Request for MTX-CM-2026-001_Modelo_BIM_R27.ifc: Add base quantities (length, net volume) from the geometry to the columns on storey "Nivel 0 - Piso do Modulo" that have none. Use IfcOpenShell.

First a look at what the model holds.

```python
import ifcopenshell
import ifcopenshell.util.element
import ifcopenshell.util.unit

model = ifcopenshell.open("MTX-CM-2026-001_Modelo_BIM_R27.ifc")
print(model.schema)
for unit_type in ("LENGTHUNIT", "AREAUNIT", "VOLUMEUNIT"):
    print(unit_type, ifcopenshell.util.unit.calculate_unit_scale(model, unit_type))
storey = next(s for s in model.by_type("IfcBuildingStorey") if s.Name == "Nivel 0 - Piso do Modulo")
columns = [e for e in ifcopenshell.util.element.get_decomposition(storey) if e.is_a("IfcColumn")]
for e in sorted(columns, key=lambda e: e.id()):
    print(e.id(), e.is_a(), e.Name, list(ifcopenshell.util.element.get_psets(e, qtos_only=True)), sep=" | ")
```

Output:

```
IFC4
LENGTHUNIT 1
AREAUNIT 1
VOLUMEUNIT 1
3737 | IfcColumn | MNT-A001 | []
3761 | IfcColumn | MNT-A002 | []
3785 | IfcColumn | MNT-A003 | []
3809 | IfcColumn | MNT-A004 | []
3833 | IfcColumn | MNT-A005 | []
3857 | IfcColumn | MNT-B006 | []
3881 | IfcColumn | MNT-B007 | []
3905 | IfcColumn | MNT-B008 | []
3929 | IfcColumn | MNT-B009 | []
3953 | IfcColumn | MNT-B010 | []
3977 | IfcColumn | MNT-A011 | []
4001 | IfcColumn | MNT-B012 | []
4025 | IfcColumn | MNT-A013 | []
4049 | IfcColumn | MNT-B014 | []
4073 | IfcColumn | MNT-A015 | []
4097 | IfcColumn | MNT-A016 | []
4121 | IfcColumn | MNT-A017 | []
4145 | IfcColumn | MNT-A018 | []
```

```python
import ifcopenshell
import ifcopenshell.api.pset
import ifcopenshell.geom
import ifcopenshell.util.element
import ifcopenshell.util.shape
import ifcopenshell.util.unit

model = ifcopenshell.open("MTX-CM-2026-001_Modelo_BIM_R27.ifc")
unit_scale = ifcopenshell.util.unit.calculate_unit_scale(model)
volume_scale = ifcopenshell.util.unit.calculate_unit_scale(model, "VOLUMEUNIT")
settings = ifcopenshell.geom.settings()

storey = next(s for s in model.by_type("IfcBuildingStorey") if s.Name == "Nivel 0 - Piso do Modulo")
columns = [e for e in ifcopenshell.util.element.get_decomposition(storey) if e.is_a("IfcColumn")]

for e in sorted(columns, key=lambda e: e.id()):
    if ifcopenshell.util.element.get_psets(e, qtos_only=True, should_inherit=False):
        continue
    # Geometry comes back in metres, in the element's own axes.
    shape = ifcopenshell.geom.create_shape(settings, e)
    values = {
        "Length": ifcopenshell.util.shape.get_z(shape.geometry) / unit_scale,
        "NetVolume": ifcopenshell.util.shape.get_volume(shape.geometry) / volume_scale,
    }
    qto = ifcopenshell.api.pset.add_qto(model, product=e, name="Qto_ColumnBaseQuantities")
    ifcopenshell.api.pset.edit_qto(model, qto=qto, properties=values)
    print(e.id(), {k: round(v, 3) for k, v in values.items()})

model.write("MTX-CM-2026-001_Modelo_BIM_R27-out.ifc")
```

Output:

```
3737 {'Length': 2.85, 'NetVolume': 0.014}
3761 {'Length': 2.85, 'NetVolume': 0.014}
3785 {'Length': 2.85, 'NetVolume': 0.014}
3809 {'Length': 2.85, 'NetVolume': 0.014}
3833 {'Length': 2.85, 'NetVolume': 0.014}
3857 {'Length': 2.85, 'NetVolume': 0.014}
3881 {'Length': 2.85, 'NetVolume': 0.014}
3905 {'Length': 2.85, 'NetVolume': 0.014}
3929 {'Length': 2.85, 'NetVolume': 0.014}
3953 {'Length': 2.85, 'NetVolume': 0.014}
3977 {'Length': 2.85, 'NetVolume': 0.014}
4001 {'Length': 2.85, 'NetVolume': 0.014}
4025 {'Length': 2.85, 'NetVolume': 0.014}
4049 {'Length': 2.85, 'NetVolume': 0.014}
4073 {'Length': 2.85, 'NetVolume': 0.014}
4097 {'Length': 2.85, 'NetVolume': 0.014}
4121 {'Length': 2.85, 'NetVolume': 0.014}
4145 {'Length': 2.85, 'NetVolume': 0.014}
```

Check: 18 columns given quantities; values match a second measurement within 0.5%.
